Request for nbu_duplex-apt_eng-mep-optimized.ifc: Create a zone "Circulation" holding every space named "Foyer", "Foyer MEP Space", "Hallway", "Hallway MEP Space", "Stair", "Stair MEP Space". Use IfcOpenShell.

First a look at what the model holds.

```python
import ifcopenshell

model = ifcopenshell.open("nbu_duplex-apt_eng-mep-optimized.ifc")
print(model.schema)
seen = {}
for space in model.by_type("IfcSpace"):
    seen[space.LongName] = seen.get(space.LongName, 0) + 1
for name, count in sorted(seen.items(), key=str):
    print(count, "x", name)
print("zones:", [z.Name for z in model.by_type("IfcZone")][:20])
```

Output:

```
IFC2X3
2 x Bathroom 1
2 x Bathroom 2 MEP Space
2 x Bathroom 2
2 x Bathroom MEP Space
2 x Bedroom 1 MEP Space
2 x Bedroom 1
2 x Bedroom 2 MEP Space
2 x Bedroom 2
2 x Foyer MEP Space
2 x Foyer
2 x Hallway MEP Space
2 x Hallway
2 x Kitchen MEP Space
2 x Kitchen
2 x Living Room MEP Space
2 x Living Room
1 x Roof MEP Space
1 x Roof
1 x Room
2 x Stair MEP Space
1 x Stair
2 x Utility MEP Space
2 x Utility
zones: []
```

```python
import ifcopenshell
import ifcopenshell.api.group
import ifcopenshell.api.root

model = ifcopenshell.open("nbu_duplex-apt_eng-mep-optimized.ifc")

names = {"Foyer", "Foyer MEP Space", "Hallway", "Hallway MEP Space", "Stair", "Stair MEP Space"}
spaces = [s for s in model.by_type("IfcSpace") if s.LongName in names]

zone = ifcopenshell.api.root.create_entity(model, ifc_class="IfcZone", name="Circulation")
ifcopenshell.api.group.assign_group(model, products=spaces, group=zone)
print(len(spaces), "spaces in", zone.Name)

model.write("nbu_duplex-apt_eng-mep-optimized_updated.ifc")
```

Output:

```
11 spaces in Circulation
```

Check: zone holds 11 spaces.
